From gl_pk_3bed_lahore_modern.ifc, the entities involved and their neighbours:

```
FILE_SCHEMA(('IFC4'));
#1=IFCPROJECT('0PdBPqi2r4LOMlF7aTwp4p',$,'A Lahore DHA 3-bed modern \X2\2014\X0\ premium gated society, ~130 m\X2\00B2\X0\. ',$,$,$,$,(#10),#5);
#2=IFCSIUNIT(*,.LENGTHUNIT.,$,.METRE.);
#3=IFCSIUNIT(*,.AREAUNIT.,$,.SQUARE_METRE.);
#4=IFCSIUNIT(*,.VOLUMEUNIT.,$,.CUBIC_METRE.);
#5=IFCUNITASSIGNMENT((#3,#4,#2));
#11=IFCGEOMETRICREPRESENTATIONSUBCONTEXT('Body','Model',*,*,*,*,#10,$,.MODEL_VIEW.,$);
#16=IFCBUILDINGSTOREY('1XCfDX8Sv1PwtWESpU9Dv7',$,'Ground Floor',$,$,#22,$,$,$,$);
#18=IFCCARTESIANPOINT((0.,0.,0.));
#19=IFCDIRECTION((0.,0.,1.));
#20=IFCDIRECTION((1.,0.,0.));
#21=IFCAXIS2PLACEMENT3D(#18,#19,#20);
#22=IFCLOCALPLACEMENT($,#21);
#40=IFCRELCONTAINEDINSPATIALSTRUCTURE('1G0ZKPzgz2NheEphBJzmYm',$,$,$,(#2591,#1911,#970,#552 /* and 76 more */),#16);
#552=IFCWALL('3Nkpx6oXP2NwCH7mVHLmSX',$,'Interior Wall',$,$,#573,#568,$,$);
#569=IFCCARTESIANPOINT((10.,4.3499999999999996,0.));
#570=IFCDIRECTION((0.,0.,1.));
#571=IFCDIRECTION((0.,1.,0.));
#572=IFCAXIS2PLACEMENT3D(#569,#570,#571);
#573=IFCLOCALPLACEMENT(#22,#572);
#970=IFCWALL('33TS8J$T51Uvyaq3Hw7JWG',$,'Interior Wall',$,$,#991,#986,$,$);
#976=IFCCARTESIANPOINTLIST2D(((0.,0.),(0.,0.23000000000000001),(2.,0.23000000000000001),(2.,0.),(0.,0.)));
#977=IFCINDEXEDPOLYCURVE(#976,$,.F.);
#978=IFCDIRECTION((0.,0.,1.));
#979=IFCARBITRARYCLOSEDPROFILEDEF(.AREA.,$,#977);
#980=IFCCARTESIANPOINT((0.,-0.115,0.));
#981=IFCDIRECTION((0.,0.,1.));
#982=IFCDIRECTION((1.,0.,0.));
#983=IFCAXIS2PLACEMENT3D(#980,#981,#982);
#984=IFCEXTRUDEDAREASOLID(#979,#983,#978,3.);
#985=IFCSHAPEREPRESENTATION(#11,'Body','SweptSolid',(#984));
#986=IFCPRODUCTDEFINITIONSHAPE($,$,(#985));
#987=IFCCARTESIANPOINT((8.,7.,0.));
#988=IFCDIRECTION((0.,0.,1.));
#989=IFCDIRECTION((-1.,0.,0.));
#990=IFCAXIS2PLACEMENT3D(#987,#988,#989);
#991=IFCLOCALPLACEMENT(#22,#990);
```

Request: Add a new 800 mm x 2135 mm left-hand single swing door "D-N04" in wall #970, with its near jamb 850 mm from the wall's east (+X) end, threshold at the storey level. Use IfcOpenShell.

```python
import numpy as np
import ifcopenshell
import ifcopenshell.api.feature
import ifcopenshell.api.geometry
import ifcopenshell.api.root
import ifcopenshell.api.spatial
import ifcopenshell.geom
import ifcopenshell.util.element
import ifcopenshell.util.placement
import ifcopenshell.util.representation
import ifcopenshell.util.shape
import ifcopenshell.util.unit

model = ifcopenshell.open("gl_pk_3bed_lahore_modern.ifc")
unit_scale = ifcopenshell.util.unit.calculate_unit_scale(model)
settings = ifcopenshell.geom.settings()


def volume(element):
    """Net volume in cubic metres, openings subtracted."""
    shape = ifcopenshell.geom.create_shape(settings, element)
    return ifcopenshell.util.shape.get_volume(shape.geometry)


wall = model.by_id(970)
storey = ifcopenshell.util.element.get_container(wall, ifc_class="IfcBuildingStorey")
context = ifcopenshell.util.representation.get_context(model, "Model", "Body", "MODEL_VIEW")
before = volume(wall)

width, height, from_end, sill = 0.8, 2.135, 0.85, 0.0  # metres

# The wall runs along its own X axis, and the end named is its -X end.
wall_shape = ifcopenshell.geom.create_shape(settings, wall)
x, y, z = ifcopenshell.util.shape.get_vertices(wall_shape.geometry).T
start = x.min() + from_end
face, thickness = float(y.min()), float(y.max() - y.min())
wall_matrix = ifcopenshell.util.placement.get_local_placement(wall.ObjectPlacement)
level = ifcopenshell.util.placement.get_local_placement(storey.ObjectPlacement)[2, 3]


def in_wall(x, y):
    """Placement at x, y metres in the wall's axes, at sill height."""
    matrix = wall_matrix.copy()
    matrix[:, 3] = wall_matrix @ np.array([x / unit_scale, y / unit_scale, 0.0, 1.0])
    matrix[2, 3] = level + sill / unit_scale
    return matrix


# Opening: a box that overshoots both wall faces by 50 mm.
opening = ifcopenshell.api.root.create_entity(model, ifc_class="IfcOpeningElement", predefined_type="OPENING")
box = ifcopenshell.api.geometry.add_wall_representation(
    model, context=context, length=width, height=height, thickness=thickness + 0.1
)
ifcopenshell.api.geometry.assign_representation(model, product=opening, representation=box)
ifcopenshell.api.geometry.edit_object_placement(model, product=opening, matrix=in_wall(start, face - 0.05), is_si=False)
ifcopenshell.api.feature.add_feature(model, feature=opening, element=wall)

door = ifcopenshell.api.root.create_entity(model, ifc_class="IfcDoor", name="D-N04", predefined_type="DOOR")
door.OverallWidth, door.OverallHeight = width / unit_scale, height / unit_scale
door.OperationType = "SINGLE_SWING_LEFT"
body = ifcopenshell.api.geometry.add_door_representation(
    model,
    context=context,
    overall_width=door.OverallWidth,
    overall_height=door.OverallHeight,
    operation_type="SINGLE_SWING_LEFT",
    lining_properties={"LiningDepth": thickness / unit_scale, "ThresholdDepth": thickness / unit_scale},
)
ifcopenshell.api.geometry.assign_representation(model, product=door, representation=body)
ifcopenshell.api.spatial.assign_container(model, products=[door], relating_structure=storey)
ifcopenshell.api.feature.add_filling(model, opening=opening, element=door)

# The lining spans the wall, so the door starts at the wall face.
ifcopenshell.api.geometry.edit_object_placement(model, product=door, matrix=in_wall(start, face), is_si=False)

after = volume(wall)

print(f"wall volume {before:.3f} -> {after:.3f} m3")

model.write("gl_pk_3bed_lahore_modern_rev.ifc")
```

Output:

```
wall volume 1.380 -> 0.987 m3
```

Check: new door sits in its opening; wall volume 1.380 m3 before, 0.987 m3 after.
